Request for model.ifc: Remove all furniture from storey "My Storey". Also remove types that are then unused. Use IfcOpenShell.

First a look at what the model holds.

```python
import ifcopenshell
import ifcopenshell.util.element

model = ifcopenshell.open("model.ifc")
print(model.schema)
storey = next(s for s in model.by_type("IfcBuildingStorey") if s.Name == "My Storey")
furniture = [e for e in ifcopenshell.util.element.get_decomposition(storey) if e.is_a("IfcFurnishingElement")]
seen = {}
for e in furniture:
    element_type = ifcopenshell.util.element.get_type(e)
    name = element_type.Name if element_type not in (None, e) else None
    seen[name] = seen.get(name, 0) + 1
for name, count in sorted(seen.items(), key=str):
    print(count, "x", name)
```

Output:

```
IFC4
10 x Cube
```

```python
import ifcopenshell
import ifcopenshell.api.root
import ifcopenshell.util.element

model = ifcopenshell.open("model.ifc")

storey = next(s for s in model.by_type("IfcBuildingStorey") if s.Name == "My Storey")
furniture = [e for e in ifcopenshell.util.element.get_decomposition(storey) if e.is_a("IfcFurnishingElement")]
types = {ifcopenshell.util.element.get_type(e) for e in furniture} - {None, *furniture}

for e in furniture:
    ifcopenshell.api.root.remove_product(model, product=e)
print(len(furniture), "removed")

unused = [t for t in types if not ifcopenshell.util.element.get_types(t)]
for t in unused:
    ifcopenshell.api.root.remove_product(model, product=t)
print(len(unused), "unused types removed")

model.write("model_v2.ifc")
```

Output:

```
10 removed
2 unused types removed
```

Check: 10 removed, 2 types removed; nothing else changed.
